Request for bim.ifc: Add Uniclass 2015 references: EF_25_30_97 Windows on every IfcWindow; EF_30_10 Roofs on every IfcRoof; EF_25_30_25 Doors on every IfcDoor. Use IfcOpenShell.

First a look at what the model holds.

```python
import ifcopenshell

model = ifcopenshell.open("bim.ifc")
print(model.schema)
print("classifications:", [c.Name for c in model.by_type("IfcClassification")])
for ifc_class in ("IfcDoor", "IfcRoof", "IfcStair", "IfcWall", "IfcWindow"):
    print(ifc_class, len(model.by_type(ifc_class)))
```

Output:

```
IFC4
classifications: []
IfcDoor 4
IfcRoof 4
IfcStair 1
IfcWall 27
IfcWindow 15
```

```python
import ifcopenshell
import ifcopenshell.api.classification

model = ifcopenshell.open("bim.ifc")

system = ifcopenshell.api.classification.add_classification(model, classification="Uniclass 2015")

codes = {
    "IfcWindow": ("EF_25_30_97", "Windows"),
    "IfcRoof": ("EF_30_10", "Roofs"),
    "IfcDoor": ("EF_25_30_25", "Doors"),
}
for ifc_class, (code, name) in codes.items():
    products = model.by_type(ifc_class)
    ifcopenshell.api.classification.add_reference(
        model, products=products, classification=system, identification=code, name=name
    )
    print(code, len(products))

model.write("bim_edited.ifc")
```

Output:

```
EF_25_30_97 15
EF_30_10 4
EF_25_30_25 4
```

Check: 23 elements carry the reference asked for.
